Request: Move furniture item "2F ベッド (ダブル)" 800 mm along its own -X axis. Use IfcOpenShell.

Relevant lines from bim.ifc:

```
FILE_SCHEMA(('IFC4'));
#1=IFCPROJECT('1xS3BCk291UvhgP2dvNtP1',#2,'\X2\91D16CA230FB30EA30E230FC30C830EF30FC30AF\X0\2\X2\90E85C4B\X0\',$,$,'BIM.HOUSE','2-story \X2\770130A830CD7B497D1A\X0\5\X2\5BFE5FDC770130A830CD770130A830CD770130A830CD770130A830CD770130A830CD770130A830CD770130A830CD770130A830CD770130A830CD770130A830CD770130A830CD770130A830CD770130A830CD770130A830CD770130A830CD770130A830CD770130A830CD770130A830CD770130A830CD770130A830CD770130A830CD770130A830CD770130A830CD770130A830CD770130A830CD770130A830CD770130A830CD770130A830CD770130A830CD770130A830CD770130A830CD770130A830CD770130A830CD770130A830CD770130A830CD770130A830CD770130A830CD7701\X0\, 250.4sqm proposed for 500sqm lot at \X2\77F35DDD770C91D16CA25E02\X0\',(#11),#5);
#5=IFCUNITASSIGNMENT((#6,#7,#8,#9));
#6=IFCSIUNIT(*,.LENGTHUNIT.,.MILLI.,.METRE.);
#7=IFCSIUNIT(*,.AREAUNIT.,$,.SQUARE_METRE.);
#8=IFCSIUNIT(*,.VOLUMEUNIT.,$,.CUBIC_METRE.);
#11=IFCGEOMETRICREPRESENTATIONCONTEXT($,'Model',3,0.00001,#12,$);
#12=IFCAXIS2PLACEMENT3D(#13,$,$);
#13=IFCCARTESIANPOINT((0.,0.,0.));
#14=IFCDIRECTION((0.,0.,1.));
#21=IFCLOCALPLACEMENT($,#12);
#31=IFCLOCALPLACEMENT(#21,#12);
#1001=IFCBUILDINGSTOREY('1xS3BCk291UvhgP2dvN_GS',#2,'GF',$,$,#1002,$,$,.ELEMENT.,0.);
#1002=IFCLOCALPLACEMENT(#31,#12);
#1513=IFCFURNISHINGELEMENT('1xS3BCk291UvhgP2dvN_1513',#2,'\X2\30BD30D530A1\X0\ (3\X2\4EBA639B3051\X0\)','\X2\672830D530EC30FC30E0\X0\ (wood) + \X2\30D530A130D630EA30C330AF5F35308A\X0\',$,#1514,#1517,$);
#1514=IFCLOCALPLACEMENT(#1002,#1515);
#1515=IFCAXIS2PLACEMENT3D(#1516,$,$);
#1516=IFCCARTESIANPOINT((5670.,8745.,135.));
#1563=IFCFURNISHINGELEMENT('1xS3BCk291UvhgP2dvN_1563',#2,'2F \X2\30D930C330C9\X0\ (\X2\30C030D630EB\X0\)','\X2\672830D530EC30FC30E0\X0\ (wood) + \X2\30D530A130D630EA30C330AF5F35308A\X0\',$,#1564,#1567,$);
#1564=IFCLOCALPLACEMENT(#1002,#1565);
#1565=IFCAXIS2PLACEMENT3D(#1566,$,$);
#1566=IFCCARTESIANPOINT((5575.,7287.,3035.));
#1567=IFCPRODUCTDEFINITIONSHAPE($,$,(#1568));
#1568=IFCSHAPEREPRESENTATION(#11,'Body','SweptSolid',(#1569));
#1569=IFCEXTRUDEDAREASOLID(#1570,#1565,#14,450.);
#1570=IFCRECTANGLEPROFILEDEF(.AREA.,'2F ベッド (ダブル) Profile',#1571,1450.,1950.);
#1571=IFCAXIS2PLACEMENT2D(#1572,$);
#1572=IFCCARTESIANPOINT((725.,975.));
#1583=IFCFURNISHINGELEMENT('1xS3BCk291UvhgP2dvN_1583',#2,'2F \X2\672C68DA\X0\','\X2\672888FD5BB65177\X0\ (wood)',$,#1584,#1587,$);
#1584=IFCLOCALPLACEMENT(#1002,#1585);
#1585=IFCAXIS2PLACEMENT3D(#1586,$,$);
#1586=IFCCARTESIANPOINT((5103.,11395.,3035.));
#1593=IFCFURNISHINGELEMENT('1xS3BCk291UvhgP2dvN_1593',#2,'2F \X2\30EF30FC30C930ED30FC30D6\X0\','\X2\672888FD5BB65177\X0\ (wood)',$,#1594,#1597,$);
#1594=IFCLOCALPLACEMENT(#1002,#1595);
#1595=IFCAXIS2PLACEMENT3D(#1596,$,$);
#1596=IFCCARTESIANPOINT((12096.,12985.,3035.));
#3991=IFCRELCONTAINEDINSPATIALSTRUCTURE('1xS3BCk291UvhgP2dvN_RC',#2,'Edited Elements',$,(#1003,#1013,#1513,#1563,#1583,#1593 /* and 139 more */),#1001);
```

```python
import ifcopenshell
import ifcopenshell.api.geometry
import ifcopenshell.util.placement

model = ifcopenshell.open("bim.ifc")

item = model.by_guid("1xS3BCk291UvhgP2dvN_1563")
matrix = ifcopenshell.util.placement.get_local_placement(item.ObjectPlacement)
matrix[:3, 3] -= matrix[:3, 0] * 800.0
ifcopenshell.api.geometry.edit_object_placement(model, product=item, matrix=matrix, is_si=False)

print(ifcopenshell.util.placement.get_local_placement(item.ObjectPlacement).round(3) + 0.0)

model.write("bim_updated.ifc")
```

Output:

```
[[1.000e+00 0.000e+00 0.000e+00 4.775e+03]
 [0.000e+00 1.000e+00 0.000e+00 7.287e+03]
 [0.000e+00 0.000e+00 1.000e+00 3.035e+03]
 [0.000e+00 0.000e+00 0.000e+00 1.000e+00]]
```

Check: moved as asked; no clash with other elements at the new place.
